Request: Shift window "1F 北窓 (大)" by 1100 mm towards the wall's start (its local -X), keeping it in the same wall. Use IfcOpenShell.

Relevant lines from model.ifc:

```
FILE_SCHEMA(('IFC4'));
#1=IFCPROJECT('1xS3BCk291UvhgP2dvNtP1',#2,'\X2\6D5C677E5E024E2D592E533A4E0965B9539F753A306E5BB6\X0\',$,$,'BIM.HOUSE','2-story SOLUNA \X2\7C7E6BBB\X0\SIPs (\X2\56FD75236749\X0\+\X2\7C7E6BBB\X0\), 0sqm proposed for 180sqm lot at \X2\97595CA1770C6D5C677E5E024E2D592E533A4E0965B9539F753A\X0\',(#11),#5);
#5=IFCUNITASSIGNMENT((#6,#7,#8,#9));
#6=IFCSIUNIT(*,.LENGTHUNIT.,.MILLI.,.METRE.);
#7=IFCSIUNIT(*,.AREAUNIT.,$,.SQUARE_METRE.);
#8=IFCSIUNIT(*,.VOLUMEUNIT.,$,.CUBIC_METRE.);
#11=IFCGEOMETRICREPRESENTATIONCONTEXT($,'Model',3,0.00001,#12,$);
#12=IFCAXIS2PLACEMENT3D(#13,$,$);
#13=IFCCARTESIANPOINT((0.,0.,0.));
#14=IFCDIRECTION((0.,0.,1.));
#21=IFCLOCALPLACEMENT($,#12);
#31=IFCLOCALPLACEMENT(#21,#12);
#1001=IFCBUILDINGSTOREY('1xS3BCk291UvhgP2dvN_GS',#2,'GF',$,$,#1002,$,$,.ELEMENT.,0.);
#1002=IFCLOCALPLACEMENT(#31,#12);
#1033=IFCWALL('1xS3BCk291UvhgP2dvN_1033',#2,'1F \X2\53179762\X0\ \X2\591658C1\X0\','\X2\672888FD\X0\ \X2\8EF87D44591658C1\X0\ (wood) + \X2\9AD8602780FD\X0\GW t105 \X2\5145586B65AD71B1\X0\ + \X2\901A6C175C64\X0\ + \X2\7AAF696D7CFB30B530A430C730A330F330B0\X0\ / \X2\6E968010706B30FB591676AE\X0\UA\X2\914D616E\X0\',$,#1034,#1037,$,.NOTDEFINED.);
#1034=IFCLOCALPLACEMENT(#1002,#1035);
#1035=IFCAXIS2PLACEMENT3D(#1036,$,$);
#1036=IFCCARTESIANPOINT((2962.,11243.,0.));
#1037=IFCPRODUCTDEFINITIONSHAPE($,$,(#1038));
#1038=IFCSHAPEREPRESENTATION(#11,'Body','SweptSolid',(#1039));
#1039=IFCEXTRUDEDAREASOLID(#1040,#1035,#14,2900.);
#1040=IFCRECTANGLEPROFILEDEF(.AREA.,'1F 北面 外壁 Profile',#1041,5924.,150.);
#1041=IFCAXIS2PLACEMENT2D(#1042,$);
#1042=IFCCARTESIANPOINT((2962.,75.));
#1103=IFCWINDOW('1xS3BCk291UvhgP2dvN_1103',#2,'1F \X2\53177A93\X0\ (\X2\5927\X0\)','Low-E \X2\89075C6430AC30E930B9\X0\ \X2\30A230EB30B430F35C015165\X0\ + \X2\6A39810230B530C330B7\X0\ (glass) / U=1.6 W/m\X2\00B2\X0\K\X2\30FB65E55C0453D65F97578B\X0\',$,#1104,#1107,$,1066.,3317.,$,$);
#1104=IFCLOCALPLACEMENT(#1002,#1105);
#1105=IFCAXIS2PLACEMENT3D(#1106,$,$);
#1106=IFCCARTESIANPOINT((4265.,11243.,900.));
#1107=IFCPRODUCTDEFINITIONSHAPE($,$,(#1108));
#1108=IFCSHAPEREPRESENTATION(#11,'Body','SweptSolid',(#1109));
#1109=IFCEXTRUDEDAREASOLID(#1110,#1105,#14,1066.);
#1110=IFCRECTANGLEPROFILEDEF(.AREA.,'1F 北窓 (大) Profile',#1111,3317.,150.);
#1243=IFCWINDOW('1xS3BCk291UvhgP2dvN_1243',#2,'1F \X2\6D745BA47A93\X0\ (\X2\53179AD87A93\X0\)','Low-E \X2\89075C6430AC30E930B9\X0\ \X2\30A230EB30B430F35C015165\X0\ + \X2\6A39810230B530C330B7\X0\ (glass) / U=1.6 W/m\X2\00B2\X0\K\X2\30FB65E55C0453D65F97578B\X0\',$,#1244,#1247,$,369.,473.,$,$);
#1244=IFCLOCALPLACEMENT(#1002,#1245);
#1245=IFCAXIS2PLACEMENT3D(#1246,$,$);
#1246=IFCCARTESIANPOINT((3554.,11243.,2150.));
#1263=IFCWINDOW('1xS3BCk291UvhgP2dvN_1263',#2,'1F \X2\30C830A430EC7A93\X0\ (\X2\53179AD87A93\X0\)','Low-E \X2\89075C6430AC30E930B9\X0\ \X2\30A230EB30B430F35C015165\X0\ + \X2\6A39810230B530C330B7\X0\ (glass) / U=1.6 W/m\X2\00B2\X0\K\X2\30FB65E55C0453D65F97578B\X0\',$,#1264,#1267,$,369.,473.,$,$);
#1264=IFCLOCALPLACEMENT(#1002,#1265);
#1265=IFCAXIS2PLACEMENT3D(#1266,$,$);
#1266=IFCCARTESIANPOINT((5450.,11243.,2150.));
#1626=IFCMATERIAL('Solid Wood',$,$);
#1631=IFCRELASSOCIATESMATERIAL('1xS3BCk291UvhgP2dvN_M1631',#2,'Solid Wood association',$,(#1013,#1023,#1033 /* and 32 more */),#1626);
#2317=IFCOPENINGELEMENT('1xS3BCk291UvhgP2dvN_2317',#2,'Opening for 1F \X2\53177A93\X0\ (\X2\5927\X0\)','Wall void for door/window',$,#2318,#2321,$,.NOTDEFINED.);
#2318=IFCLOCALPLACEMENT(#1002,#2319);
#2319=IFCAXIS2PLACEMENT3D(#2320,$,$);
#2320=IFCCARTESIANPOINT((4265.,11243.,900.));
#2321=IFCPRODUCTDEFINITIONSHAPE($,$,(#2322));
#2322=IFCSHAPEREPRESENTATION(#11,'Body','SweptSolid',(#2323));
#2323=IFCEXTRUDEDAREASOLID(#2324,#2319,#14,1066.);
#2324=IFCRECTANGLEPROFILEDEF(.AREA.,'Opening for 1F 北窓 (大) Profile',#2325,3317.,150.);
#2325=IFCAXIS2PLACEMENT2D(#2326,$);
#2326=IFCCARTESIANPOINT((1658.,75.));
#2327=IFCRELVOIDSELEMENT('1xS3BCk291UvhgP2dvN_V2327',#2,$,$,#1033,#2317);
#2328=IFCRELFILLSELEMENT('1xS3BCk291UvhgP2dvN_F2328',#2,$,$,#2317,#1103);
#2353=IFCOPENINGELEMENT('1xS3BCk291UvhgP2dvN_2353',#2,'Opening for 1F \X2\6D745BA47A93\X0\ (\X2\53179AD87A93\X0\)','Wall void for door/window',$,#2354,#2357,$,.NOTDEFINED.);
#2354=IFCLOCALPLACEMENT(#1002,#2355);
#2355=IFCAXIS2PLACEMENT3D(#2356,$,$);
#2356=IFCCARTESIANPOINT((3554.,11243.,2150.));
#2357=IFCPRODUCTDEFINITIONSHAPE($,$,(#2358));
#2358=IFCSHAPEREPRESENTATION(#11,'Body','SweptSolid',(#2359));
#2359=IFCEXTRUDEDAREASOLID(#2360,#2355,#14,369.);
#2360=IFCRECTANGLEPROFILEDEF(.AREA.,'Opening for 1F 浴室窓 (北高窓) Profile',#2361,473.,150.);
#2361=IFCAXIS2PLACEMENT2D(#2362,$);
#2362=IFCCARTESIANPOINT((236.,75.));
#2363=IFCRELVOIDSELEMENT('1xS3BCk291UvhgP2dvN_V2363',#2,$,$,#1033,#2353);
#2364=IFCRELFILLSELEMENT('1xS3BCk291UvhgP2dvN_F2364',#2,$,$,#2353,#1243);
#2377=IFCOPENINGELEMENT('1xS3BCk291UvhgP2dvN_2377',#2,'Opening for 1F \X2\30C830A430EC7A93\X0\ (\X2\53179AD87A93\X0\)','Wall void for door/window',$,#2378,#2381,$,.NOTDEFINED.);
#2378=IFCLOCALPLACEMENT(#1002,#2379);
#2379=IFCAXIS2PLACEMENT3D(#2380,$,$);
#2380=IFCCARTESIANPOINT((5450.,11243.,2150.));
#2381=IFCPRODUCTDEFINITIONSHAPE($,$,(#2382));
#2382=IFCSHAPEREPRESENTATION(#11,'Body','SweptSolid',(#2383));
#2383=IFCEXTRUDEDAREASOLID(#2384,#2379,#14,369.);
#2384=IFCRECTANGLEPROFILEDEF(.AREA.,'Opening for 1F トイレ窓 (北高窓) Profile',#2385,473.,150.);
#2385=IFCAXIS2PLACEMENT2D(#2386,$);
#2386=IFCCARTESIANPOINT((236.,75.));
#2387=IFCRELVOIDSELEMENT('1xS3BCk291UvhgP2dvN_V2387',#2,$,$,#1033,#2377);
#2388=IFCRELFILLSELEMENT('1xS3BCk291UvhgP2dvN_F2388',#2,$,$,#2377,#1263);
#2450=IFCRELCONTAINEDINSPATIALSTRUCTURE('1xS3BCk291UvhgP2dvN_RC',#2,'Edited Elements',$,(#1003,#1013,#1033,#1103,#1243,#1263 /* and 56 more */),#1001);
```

```python
import ifcopenshell
import ifcopenshell.api.geometry
import ifcopenshell.util.placement
import ifcopenshell.util.unit

model = ifcopenshell.open("model.ifc")
unit_scale = ifcopenshell.util.unit.calculate_unit_scale(model)

window = model.by_guid("1xS3BCk291UvhgP2dvN_1103")
opening = window.FillsVoids[0].RelatingOpeningElement
wall = opening.VoidsElements[0].RelatingBuildingElement

wall_matrix = ifcopenshell.util.placement.get_local_placement(wall.ObjectPlacement)
shift = wall_matrix[:3, 0] * -1.1 / unit_scale
before = ifcopenshell.util.placement.get_local_placement(window.ObjectPlacement)[:3, 3].copy()

# The window is not placed relative to its opening, so move both.
for product in (opening, window):
    matrix = ifcopenshell.util.placement.get_local_placement(product.ObjectPlacement)
    matrix[:3, 3] += shift
    ifcopenshell.api.geometry.edit_object_placement(model, product=product, matrix=matrix, is_si=False)

after = ifcopenshell.util.placement.get_local_placement(window.ObjectPlacement)[:3, 3]
print("window moved by", (after - before).round(3) + 0.0)

model.write("model_rev.ifc")
```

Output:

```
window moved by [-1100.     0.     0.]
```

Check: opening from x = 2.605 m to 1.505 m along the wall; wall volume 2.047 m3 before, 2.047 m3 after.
